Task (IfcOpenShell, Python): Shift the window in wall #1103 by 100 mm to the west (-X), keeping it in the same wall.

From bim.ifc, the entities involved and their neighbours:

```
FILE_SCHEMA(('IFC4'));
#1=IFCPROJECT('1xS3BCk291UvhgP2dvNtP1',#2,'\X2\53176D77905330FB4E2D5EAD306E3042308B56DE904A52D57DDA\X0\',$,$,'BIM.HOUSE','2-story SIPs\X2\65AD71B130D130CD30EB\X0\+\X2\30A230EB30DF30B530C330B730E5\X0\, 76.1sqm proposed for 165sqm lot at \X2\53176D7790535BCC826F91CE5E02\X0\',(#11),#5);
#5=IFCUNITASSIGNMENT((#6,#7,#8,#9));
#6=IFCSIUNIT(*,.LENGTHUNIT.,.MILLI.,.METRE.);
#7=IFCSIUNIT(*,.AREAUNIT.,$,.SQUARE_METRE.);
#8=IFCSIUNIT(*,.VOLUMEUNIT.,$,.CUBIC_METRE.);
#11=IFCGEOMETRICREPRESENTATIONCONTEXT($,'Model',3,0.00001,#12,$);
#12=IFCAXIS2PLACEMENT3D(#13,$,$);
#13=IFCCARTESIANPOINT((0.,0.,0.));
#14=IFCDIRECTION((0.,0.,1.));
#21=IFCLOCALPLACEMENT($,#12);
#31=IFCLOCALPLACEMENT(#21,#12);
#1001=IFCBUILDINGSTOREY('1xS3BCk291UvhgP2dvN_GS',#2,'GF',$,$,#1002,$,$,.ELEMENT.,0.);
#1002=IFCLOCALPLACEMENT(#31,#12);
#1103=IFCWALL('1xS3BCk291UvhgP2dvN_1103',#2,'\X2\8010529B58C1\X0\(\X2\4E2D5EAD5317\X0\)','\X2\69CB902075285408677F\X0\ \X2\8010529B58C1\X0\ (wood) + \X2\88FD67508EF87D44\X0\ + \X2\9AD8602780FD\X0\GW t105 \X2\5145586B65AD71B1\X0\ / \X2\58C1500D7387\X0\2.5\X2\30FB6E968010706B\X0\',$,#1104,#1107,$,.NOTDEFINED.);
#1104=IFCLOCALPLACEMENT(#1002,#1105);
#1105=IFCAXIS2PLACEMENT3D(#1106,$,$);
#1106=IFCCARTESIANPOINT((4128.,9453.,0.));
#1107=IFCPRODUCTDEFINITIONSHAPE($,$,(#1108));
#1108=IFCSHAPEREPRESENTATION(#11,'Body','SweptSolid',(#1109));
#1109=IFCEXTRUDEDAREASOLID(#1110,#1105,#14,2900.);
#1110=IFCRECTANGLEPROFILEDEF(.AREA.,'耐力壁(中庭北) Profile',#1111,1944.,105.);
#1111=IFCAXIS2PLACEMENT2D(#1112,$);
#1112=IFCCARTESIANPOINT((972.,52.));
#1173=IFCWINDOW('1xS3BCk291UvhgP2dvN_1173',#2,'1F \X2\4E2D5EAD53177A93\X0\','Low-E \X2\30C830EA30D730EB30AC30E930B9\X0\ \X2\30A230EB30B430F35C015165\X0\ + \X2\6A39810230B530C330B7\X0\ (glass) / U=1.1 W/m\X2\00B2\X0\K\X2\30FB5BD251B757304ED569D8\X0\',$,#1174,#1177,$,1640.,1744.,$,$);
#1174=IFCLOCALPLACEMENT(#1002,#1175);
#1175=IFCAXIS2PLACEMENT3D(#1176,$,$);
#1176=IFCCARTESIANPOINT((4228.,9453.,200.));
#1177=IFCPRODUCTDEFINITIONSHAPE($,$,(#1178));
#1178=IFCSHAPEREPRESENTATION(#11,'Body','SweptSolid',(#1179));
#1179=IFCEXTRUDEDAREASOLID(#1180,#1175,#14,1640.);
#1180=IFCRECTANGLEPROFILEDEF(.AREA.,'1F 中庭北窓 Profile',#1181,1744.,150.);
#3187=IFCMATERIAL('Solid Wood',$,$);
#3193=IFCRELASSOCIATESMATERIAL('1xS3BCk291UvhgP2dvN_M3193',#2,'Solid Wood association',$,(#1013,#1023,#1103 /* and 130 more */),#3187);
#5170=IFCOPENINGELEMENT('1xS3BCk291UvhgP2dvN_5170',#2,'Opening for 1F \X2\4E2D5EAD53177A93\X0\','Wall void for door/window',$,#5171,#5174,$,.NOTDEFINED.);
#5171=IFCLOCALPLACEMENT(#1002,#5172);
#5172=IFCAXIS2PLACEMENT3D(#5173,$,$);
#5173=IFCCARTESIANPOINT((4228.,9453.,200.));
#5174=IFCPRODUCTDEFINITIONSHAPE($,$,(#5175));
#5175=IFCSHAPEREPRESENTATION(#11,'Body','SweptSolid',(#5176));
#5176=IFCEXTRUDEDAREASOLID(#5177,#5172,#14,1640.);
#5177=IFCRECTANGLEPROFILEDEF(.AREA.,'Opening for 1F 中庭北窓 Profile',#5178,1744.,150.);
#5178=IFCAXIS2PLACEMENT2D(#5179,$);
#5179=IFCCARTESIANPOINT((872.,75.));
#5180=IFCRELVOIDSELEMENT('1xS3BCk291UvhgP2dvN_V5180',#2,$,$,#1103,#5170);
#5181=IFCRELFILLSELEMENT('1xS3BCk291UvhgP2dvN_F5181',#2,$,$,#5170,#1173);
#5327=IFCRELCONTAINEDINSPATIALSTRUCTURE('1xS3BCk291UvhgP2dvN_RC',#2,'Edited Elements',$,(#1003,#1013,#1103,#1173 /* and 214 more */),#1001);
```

```python
import ifcopenshell
import ifcopenshell.api.geometry
import ifcopenshell.util.placement
import ifcopenshell.util.unit

model = ifcopenshell.open("bim.ifc")
unit_scale = ifcopenshell.util.unit.calculate_unit_scale(model)

window = model.by_guid("1xS3BCk291UvhgP2dvN_1173")
opening = window.FillsVoids[0].RelatingOpeningElement
wall = opening.VoidsElements[0].RelatingBuildingElement

wall_matrix = ifcopenshell.util.placement.get_local_placement(wall.ObjectPlacement)
shift = wall_matrix[:3, 0] * -0.1 / unit_scale
before = ifcopenshell.util.placement.get_local_placement(window.ObjectPlacement)[:3, 3].copy()

# The window is not placed relative to its opening, so move both.
for product in (opening, window):
    matrix = ifcopenshell.util.placement.get_local_placement(product.ObjectPlacement)
    matrix[:3, 3] += shift
    ifcopenshell.api.geometry.edit_object_placement(model, product=product, matrix=matrix, is_si=False)

after = ifcopenshell.util.placement.get_local_placement(window.ObjectPlacement)[:3, 3]
print("window moved by", (after - before).round(3) + 0.0)

model.write("bim_edited.ifc")
```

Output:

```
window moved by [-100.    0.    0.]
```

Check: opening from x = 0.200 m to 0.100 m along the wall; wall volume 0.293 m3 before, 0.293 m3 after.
